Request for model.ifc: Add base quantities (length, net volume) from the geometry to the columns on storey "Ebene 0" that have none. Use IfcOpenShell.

First a look at what the model holds.

```python
import ifcopenshell
import ifcopenshell.util.element
import ifcopenshell.util.unit

model = ifcopenshell.open("model.ifc")
print(model.schema)
for unit_type in ("LENGTHUNIT", "AREAUNIT", "VOLUMEUNIT"):
    print(unit_type, ifcopenshell.util.unit.calculate_unit_scale(model, unit_type))
storey = next(s for s in model.by_type("IfcBuildingStorey") if s.Name == "Ebene 0")
columns = [e for e in ifcopenshell.util.element.get_decomposition(storey) if e.is_a("IfcColumn")]
for e in sorted(columns, key=lambda e: e.id()):
    print(e.id(), e.is_a(), e.Name, list(ifcopenshell.util.element.get_psets(e, qtos_only=True)), sep=" | ")
```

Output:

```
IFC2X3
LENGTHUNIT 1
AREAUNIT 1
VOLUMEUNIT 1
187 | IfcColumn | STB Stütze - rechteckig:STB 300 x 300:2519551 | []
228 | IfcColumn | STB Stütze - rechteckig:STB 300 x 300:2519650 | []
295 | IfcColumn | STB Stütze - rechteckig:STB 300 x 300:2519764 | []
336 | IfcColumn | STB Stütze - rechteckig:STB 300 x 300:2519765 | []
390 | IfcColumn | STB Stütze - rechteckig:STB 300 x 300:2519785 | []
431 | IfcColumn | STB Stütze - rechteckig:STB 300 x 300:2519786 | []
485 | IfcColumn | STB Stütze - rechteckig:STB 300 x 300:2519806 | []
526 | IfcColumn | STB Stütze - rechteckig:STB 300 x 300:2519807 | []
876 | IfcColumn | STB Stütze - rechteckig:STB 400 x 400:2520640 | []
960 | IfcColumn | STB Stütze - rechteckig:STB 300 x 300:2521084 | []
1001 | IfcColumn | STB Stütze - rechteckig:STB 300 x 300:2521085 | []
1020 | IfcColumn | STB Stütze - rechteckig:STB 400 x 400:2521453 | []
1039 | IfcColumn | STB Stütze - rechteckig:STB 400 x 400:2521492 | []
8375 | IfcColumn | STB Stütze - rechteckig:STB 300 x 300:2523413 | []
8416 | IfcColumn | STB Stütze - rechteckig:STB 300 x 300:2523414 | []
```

```python
import ifcopenshell
import ifcopenshell.api.pset
import ifcopenshell.geom
import ifcopenshell.util.element
import ifcopenshell.util.shape
import ifcopenshell.util.unit

model = ifcopenshell.open("model.ifc")
unit_scale = ifcopenshell.util.unit.calculate_unit_scale(model)
volume_scale = ifcopenshell.util.unit.calculate_unit_scale(model, "VOLUMEUNIT")
settings = ifcopenshell.geom.settings()

storey = next(s for s in model.by_type("IfcBuildingStorey") if s.Name == "Ebene 0")
columns = [e for e in ifcopenshell.util.element.get_decomposition(storey) if e.is_a("IfcColumn")]

for e in sorted(columns, key=lambda e: e.id()):
    if ifcopenshell.util.element.get_psets(e, qtos_only=True, should_inherit=False):
        continue
    # Geometry comes back in metres, in the element's own axes.
    shape = ifcopenshell.geom.create_shape(settings, e)
    values = {
        "Length": ifcopenshell.util.shape.get_z(shape.geometry) / unit_scale,
        "NetVolume": ifcopenshell.util.shape.get_volume(shape.geometry) / volume_scale,
    }
    qto = ifcopenshell.api.pset.add_qto(model, product=e, name="BaseQuantities")
    ifcopenshell.api.pset.edit_qto(model, qto=qto, properties=values)
    print(e.id(), {k: round(v, 3) for k, v in values.items()})

model.write("model_v2.ifc")
```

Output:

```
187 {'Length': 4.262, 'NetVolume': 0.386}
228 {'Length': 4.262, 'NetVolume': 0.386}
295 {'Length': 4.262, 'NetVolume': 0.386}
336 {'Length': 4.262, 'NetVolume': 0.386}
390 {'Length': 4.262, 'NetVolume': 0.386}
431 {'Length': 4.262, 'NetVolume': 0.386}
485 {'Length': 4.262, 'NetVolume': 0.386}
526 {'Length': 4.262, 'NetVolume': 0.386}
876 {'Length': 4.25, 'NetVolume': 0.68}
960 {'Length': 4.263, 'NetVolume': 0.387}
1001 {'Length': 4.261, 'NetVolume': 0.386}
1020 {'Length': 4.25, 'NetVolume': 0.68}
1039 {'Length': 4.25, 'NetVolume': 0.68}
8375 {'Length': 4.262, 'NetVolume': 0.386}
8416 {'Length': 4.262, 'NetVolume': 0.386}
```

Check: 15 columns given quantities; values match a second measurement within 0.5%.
